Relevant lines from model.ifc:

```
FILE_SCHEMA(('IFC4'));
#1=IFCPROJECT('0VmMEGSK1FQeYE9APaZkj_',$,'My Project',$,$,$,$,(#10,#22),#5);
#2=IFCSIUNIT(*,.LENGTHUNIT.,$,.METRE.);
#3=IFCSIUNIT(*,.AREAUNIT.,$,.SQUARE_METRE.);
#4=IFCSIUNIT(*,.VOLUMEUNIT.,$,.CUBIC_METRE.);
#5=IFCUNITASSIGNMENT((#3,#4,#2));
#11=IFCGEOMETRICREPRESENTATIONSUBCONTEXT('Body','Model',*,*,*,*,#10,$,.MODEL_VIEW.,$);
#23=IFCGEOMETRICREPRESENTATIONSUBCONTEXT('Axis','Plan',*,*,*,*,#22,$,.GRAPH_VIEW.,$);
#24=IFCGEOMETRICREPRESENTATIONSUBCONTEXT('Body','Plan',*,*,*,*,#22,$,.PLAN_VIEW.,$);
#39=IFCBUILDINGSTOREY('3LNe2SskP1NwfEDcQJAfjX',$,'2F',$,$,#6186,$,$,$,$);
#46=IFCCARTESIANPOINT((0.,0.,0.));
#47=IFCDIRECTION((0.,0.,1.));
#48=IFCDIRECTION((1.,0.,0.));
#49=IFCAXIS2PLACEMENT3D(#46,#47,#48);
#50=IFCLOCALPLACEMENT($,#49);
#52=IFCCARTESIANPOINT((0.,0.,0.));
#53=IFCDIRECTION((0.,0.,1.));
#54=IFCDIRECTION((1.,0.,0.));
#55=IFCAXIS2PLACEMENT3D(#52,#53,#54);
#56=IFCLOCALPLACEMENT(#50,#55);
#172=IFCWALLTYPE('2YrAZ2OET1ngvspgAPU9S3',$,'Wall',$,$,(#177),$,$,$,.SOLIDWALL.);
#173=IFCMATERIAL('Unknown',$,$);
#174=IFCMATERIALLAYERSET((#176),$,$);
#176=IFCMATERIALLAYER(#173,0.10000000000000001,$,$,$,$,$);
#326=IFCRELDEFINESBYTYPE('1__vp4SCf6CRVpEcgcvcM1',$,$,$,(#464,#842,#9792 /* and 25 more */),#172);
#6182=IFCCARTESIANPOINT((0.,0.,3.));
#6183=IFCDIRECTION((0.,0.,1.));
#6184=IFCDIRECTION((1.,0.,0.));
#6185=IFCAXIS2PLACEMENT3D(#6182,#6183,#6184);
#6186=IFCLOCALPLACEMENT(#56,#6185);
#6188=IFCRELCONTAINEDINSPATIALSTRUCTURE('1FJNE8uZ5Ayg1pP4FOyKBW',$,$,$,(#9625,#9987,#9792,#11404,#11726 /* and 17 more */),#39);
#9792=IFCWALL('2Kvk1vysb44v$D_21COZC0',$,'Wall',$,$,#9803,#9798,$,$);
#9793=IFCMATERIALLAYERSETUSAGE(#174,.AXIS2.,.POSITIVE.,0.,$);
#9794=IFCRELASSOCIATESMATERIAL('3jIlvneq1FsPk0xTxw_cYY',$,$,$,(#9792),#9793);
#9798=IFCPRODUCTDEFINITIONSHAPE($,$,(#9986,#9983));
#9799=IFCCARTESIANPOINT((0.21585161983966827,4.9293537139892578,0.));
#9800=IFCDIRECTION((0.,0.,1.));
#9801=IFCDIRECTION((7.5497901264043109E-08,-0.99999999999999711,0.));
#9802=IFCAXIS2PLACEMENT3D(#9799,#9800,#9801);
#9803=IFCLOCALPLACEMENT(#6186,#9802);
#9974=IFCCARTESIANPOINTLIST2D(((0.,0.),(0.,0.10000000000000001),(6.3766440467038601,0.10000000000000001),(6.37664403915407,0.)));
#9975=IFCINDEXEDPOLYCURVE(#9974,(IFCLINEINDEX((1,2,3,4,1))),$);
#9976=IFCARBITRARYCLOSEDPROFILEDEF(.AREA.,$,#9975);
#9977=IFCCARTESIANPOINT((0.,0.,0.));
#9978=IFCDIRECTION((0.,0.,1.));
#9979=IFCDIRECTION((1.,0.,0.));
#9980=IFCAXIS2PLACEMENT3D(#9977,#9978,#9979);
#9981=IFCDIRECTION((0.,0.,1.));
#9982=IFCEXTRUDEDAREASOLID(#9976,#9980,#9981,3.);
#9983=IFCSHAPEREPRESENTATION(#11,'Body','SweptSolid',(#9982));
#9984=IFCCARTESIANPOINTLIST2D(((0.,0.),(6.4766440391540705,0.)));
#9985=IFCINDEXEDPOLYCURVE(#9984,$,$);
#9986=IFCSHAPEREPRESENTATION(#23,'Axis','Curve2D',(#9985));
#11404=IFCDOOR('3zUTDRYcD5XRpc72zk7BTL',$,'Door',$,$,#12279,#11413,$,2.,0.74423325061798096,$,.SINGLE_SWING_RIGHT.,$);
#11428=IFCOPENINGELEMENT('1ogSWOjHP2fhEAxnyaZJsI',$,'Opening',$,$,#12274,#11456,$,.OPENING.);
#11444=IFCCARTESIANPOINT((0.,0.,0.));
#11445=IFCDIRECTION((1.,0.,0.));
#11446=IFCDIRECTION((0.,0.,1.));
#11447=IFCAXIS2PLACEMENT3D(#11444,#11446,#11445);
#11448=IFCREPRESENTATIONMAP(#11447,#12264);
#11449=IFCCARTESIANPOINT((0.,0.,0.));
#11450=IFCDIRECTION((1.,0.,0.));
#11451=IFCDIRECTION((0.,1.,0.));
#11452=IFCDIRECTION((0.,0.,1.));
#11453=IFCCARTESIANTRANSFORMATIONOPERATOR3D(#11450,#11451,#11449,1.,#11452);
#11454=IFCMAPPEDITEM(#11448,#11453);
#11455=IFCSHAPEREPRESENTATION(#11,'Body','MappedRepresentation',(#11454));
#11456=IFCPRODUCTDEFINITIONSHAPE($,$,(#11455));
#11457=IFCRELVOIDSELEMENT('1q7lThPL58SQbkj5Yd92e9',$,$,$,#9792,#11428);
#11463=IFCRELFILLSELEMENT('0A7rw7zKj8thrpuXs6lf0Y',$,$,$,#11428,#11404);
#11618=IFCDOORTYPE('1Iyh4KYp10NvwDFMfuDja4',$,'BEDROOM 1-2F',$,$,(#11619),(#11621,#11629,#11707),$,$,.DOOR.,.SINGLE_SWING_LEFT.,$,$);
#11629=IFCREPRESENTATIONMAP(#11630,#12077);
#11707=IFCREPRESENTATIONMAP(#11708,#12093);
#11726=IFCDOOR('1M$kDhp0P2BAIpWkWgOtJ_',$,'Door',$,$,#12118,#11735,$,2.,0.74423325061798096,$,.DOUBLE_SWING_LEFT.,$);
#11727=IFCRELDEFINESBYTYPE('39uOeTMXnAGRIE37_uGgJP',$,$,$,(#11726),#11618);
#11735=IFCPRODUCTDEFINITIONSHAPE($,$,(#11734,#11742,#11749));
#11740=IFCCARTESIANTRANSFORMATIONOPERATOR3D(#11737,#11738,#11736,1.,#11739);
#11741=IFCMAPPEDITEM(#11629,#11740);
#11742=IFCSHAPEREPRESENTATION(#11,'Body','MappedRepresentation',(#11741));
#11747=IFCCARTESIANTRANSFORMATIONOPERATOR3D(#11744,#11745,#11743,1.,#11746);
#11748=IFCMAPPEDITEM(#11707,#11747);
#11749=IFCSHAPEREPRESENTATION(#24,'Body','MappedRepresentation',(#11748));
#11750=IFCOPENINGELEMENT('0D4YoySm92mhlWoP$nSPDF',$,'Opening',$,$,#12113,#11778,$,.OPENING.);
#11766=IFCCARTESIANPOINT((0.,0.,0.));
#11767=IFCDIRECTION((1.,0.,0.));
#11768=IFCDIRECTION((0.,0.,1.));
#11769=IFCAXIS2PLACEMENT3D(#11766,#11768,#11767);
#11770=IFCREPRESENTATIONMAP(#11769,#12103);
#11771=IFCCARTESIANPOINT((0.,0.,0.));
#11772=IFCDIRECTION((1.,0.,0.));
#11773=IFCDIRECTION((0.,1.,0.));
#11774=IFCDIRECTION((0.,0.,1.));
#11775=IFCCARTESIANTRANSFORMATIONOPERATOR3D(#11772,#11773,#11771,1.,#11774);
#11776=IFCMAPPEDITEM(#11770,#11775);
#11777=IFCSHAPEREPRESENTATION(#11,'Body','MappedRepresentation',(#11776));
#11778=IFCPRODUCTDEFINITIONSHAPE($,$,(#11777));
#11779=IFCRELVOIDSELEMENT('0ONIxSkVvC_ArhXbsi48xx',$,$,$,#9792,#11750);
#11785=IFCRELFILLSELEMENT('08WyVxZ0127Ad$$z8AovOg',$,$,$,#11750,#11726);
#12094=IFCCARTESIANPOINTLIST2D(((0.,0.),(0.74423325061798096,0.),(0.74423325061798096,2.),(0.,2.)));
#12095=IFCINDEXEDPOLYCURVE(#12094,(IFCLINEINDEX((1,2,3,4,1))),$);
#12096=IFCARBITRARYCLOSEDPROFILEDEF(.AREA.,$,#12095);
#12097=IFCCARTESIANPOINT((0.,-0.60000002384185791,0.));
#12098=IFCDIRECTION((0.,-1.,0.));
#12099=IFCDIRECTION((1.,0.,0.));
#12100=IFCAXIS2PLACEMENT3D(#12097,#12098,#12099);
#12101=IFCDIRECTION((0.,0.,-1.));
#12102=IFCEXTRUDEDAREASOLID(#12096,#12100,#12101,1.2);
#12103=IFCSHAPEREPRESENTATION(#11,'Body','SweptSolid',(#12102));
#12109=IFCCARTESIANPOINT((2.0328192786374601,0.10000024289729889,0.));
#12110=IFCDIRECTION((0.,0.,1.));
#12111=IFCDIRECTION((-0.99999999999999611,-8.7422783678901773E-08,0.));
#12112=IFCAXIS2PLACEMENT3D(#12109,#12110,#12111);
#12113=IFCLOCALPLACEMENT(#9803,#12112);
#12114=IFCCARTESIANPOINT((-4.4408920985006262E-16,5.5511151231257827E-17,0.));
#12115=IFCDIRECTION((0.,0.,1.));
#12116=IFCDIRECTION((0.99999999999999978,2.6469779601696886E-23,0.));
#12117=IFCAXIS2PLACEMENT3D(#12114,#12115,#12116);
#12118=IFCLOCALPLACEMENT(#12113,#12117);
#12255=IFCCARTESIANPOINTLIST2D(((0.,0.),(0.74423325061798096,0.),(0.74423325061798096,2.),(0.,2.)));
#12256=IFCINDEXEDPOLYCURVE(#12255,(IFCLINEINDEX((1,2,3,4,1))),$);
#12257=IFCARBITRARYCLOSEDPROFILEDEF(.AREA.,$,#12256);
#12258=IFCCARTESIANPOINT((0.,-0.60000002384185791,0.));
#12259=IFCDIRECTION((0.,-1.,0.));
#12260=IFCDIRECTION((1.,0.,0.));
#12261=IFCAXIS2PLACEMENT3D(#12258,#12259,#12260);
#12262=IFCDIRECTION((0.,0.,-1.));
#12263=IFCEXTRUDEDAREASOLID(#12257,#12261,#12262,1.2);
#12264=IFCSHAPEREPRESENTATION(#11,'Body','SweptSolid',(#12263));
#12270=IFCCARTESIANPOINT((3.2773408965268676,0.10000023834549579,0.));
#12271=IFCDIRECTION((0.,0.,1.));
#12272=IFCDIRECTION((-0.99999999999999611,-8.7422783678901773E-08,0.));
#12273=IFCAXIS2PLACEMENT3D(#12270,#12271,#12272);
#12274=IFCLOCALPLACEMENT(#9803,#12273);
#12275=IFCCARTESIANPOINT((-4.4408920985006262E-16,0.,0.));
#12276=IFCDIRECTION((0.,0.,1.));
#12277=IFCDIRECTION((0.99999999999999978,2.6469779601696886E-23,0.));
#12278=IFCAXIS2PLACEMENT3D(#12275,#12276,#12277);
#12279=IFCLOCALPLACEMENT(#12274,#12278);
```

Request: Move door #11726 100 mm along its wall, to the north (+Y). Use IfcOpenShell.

```python
import ifcopenshell
import ifcopenshell.api.geometry
import ifcopenshell.util.placement
import ifcopenshell.util.unit

model = ifcopenshell.open("model.ifc")
unit_scale = ifcopenshell.util.unit.calculate_unit_scale(model)

door = model.by_id(11726)
opening = door.FillsVoids[0].RelatingOpeningElement
wall = opening.VoidsElements[0].RelatingBuildingElement

wall_matrix = ifcopenshell.util.placement.get_local_placement(wall.ObjectPlacement)
shift = wall_matrix[:3, 0] * -0.1 / unit_scale
before = ifcopenshell.util.placement.get_local_placement(door.ObjectPlacement)[:3, 3].copy()

# The door is placed relative to its opening, so it follows when the opening moves.
matrix = ifcopenshell.util.placement.get_local_placement(opening.ObjectPlacement)
matrix[:3, 3] += shift
ifcopenshell.api.geometry.edit_object_placement(
    model, product=opening, matrix=matrix, is_si=False, should_transform_children=True
)

after = ifcopenshell.util.placement.get_local_placement(door.ObjectPlacement)[:3, 3]
print("door moved by", (after - before).round(3) + 0.0)

model.write("model_rev.ifc")
```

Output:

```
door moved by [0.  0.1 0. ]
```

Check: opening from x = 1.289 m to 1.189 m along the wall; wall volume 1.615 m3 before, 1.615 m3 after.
